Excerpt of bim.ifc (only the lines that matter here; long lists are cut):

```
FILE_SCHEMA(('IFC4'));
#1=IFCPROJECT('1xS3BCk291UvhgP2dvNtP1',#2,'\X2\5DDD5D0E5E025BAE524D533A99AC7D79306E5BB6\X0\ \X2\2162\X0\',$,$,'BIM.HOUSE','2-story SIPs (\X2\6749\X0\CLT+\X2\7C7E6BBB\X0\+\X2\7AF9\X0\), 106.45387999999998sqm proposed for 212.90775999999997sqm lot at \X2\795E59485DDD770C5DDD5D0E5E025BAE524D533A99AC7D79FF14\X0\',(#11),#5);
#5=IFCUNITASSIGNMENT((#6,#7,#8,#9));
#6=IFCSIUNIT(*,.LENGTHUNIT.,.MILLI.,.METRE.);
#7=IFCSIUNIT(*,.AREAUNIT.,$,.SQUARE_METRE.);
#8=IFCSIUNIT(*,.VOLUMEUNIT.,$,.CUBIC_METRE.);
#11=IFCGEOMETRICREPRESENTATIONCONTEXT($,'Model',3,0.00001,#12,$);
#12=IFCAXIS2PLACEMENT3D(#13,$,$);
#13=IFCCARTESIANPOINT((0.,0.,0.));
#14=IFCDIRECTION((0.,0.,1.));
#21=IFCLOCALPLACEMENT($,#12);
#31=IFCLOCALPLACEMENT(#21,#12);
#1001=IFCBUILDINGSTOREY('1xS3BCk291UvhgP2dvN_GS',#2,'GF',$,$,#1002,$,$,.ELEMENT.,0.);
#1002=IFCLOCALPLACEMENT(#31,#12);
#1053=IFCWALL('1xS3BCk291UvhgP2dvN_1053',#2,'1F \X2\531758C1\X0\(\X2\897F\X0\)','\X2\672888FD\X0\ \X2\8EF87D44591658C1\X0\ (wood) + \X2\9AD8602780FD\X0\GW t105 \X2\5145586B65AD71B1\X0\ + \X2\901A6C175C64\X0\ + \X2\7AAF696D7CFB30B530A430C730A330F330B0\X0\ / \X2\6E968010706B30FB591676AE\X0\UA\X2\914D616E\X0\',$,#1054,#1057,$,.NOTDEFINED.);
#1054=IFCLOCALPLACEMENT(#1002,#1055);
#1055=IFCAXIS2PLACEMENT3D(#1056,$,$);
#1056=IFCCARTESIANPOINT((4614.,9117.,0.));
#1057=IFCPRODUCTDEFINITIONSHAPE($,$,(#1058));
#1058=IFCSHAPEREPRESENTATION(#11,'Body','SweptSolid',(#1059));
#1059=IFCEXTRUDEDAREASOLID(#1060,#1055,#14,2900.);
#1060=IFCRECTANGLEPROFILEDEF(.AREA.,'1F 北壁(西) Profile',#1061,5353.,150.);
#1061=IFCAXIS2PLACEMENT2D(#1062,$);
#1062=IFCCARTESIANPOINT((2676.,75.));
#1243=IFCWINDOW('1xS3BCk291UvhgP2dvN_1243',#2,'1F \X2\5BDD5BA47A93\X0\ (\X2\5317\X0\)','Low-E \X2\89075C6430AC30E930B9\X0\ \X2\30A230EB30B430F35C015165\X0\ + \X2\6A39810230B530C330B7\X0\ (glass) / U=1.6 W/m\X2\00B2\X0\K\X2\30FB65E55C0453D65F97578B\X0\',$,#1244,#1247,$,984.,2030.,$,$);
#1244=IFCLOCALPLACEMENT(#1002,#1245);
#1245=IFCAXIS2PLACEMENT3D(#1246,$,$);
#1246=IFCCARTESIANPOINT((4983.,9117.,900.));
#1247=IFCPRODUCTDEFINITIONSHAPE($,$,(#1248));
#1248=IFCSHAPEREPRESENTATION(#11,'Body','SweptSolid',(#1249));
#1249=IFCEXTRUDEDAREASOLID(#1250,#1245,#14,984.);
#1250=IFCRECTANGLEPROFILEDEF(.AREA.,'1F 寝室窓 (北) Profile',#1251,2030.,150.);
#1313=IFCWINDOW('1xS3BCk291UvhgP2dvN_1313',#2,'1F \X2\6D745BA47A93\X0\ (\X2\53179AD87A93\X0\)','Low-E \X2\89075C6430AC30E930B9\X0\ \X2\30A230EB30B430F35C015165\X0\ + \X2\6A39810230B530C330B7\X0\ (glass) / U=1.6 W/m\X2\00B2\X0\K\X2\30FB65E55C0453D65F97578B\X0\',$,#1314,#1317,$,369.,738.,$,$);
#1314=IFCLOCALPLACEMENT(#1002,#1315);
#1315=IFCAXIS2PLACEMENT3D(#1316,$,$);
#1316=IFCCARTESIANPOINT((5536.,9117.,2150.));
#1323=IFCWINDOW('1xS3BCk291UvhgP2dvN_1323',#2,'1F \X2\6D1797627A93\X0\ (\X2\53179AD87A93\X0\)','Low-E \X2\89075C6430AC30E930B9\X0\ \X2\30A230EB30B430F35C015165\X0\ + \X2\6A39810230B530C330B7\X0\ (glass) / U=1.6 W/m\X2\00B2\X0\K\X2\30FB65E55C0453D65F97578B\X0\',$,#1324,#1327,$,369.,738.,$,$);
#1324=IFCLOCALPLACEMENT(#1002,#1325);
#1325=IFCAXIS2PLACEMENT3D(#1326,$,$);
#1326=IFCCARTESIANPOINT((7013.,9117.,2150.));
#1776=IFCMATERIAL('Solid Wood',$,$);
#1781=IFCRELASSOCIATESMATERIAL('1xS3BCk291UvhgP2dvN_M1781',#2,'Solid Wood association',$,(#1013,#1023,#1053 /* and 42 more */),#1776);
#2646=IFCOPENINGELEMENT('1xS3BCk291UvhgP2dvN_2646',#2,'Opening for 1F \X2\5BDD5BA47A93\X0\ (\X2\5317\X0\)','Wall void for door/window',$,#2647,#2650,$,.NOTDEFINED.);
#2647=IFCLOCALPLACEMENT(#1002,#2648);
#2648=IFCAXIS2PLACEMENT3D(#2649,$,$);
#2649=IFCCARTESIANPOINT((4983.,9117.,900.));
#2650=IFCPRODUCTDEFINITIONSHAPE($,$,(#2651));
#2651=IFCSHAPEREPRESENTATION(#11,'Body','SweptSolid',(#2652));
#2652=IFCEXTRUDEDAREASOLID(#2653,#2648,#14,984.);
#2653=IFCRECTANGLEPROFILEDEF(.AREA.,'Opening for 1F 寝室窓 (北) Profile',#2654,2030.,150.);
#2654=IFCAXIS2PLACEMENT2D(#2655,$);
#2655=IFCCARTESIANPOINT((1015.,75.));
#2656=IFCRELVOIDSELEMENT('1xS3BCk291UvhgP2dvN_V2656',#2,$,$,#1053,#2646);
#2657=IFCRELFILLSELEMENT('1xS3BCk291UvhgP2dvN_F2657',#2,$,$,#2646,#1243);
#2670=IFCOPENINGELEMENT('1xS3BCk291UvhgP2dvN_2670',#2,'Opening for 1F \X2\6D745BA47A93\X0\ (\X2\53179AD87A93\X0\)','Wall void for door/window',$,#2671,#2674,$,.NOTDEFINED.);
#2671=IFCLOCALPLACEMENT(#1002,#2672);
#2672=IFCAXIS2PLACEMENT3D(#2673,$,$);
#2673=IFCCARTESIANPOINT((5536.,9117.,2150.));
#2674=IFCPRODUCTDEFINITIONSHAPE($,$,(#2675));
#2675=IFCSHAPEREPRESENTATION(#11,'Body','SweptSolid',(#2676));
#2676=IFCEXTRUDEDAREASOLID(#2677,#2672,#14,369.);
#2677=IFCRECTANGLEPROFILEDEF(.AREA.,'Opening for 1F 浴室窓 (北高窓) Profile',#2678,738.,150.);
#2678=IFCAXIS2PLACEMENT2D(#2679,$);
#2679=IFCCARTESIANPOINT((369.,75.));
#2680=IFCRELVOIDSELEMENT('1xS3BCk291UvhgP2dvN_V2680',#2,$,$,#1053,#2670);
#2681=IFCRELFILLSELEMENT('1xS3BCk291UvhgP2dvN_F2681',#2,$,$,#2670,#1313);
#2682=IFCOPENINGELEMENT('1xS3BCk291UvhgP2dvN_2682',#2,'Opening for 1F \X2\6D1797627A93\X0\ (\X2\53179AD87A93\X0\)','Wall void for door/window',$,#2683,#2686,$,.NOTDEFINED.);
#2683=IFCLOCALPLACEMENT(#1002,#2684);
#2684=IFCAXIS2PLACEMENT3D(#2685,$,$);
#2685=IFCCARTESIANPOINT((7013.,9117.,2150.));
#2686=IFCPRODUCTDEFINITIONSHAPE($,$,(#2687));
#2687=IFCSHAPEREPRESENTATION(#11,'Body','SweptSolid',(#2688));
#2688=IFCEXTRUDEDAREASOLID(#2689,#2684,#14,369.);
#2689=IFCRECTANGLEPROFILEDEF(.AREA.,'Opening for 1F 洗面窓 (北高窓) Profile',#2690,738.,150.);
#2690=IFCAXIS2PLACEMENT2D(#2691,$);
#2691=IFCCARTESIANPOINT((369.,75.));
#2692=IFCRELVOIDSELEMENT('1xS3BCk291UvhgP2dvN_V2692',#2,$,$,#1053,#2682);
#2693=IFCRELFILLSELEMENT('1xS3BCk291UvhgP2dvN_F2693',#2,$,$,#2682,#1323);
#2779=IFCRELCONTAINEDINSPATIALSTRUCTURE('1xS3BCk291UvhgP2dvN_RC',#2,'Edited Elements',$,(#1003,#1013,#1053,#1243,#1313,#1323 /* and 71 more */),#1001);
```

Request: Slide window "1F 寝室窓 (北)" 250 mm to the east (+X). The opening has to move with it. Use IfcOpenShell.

```python
import ifcopenshell
import ifcopenshell.api.geometry
import ifcopenshell.util.placement

model = ifcopenshell.open("bim.ifc")

window = model.by_id(1243)
opening = window.FillsVoids[0].RelatingOpeningElement
wall = opening.VoidsElements[0].RelatingBuildingElement

wall_matrix = ifcopenshell.util.placement.get_local_placement(wall.ObjectPlacement)
shift = wall_matrix[:3, 0] * 250.0
before = ifcopenshell.util.placement.get_local_placement(window.ObjectPlacement)[:3, 3].copy()

# The window is not placed relative to its opening, so move both.
for product in (opening, window):
    matrix = ifcopenshell.util.placement.get_local_placement(product.ObjectPlacement)
    matrix[:3, 3] += shift
    ifcopenshell.api.geometry.edit_object_placement(model, product=product, matrix=matrix, is_si=False)

after = ifcopenshell.util.placement.get_local_placement(window.ObjectPlacement)[:3, 3]
print("window moved by", (after - before).round(3) + 0.0)

model.write("bim_rev.ifc")
```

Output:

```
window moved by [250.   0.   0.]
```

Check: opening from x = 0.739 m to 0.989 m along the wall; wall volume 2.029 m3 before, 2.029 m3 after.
